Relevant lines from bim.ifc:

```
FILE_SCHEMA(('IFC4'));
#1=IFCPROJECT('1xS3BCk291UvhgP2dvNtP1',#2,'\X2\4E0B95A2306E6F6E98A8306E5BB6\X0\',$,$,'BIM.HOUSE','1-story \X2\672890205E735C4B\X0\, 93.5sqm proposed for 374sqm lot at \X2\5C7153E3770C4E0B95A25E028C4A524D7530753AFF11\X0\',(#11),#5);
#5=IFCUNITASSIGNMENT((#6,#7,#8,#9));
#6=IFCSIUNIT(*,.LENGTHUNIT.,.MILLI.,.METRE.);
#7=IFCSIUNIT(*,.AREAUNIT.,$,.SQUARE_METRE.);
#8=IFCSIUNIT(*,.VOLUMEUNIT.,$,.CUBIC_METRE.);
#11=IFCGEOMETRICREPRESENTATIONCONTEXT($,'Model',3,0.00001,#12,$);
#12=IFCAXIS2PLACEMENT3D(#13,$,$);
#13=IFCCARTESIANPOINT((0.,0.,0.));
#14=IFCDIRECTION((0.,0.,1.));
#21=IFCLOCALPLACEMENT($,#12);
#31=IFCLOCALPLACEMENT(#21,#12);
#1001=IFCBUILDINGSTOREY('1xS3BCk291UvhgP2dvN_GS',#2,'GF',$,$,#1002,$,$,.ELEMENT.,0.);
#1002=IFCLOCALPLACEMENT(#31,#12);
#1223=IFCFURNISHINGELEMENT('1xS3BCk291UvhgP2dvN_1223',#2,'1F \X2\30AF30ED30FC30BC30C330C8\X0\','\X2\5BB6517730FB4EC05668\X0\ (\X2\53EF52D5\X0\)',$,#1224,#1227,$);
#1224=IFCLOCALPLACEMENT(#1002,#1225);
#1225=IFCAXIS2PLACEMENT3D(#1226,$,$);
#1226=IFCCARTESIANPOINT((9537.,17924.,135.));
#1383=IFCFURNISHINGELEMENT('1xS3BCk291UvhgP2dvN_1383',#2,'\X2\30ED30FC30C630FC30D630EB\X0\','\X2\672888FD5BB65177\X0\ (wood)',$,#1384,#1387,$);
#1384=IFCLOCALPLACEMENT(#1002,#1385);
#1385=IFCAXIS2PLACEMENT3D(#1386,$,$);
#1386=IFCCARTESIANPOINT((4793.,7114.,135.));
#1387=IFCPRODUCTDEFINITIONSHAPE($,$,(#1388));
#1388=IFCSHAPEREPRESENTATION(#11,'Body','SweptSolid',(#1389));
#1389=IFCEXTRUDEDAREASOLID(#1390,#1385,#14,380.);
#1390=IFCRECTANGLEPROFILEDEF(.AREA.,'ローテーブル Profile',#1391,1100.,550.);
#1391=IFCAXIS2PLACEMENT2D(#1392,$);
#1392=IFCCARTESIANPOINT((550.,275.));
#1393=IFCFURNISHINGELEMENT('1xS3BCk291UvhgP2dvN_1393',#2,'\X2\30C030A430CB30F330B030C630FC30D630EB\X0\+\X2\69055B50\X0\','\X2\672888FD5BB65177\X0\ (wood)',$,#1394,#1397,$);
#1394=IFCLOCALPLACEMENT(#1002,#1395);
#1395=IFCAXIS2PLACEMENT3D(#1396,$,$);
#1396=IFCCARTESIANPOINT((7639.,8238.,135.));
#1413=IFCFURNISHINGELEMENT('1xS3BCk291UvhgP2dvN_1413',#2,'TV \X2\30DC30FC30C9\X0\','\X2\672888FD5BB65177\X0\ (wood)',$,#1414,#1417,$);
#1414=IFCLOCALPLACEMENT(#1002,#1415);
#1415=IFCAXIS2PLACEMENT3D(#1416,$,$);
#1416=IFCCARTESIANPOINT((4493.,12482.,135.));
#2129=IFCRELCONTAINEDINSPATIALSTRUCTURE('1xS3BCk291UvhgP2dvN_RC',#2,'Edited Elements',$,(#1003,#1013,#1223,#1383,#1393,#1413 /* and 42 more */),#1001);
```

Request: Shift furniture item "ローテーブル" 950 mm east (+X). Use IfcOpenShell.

```python
import ifcopenshell
import ifcopenshell.api.geometry
import ifcopenshell.util.placement

model = ifcopenshell.open("bim.ifc")

item = model.by_guid("1xS3BCk291UvhgP2dvN_1383")
matrix = ifcopenshell.util.placement.get_local_placement(item.ObjectPlacement)
matrix[0, 3] += 950.0
ifcopenshell.api.geometry.edit_object_placement(model, product=item, matrix=matrix, is_si=False)

print(ifcopenshell.util.placement.get_local_placement(item.ObjectPlacement).round(3) + 0.0)

model.write("bim-out.ifc")
```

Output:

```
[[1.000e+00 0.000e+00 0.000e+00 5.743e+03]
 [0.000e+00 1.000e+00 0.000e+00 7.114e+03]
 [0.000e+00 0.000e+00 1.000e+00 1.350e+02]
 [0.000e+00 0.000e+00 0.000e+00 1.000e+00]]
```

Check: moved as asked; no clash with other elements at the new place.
